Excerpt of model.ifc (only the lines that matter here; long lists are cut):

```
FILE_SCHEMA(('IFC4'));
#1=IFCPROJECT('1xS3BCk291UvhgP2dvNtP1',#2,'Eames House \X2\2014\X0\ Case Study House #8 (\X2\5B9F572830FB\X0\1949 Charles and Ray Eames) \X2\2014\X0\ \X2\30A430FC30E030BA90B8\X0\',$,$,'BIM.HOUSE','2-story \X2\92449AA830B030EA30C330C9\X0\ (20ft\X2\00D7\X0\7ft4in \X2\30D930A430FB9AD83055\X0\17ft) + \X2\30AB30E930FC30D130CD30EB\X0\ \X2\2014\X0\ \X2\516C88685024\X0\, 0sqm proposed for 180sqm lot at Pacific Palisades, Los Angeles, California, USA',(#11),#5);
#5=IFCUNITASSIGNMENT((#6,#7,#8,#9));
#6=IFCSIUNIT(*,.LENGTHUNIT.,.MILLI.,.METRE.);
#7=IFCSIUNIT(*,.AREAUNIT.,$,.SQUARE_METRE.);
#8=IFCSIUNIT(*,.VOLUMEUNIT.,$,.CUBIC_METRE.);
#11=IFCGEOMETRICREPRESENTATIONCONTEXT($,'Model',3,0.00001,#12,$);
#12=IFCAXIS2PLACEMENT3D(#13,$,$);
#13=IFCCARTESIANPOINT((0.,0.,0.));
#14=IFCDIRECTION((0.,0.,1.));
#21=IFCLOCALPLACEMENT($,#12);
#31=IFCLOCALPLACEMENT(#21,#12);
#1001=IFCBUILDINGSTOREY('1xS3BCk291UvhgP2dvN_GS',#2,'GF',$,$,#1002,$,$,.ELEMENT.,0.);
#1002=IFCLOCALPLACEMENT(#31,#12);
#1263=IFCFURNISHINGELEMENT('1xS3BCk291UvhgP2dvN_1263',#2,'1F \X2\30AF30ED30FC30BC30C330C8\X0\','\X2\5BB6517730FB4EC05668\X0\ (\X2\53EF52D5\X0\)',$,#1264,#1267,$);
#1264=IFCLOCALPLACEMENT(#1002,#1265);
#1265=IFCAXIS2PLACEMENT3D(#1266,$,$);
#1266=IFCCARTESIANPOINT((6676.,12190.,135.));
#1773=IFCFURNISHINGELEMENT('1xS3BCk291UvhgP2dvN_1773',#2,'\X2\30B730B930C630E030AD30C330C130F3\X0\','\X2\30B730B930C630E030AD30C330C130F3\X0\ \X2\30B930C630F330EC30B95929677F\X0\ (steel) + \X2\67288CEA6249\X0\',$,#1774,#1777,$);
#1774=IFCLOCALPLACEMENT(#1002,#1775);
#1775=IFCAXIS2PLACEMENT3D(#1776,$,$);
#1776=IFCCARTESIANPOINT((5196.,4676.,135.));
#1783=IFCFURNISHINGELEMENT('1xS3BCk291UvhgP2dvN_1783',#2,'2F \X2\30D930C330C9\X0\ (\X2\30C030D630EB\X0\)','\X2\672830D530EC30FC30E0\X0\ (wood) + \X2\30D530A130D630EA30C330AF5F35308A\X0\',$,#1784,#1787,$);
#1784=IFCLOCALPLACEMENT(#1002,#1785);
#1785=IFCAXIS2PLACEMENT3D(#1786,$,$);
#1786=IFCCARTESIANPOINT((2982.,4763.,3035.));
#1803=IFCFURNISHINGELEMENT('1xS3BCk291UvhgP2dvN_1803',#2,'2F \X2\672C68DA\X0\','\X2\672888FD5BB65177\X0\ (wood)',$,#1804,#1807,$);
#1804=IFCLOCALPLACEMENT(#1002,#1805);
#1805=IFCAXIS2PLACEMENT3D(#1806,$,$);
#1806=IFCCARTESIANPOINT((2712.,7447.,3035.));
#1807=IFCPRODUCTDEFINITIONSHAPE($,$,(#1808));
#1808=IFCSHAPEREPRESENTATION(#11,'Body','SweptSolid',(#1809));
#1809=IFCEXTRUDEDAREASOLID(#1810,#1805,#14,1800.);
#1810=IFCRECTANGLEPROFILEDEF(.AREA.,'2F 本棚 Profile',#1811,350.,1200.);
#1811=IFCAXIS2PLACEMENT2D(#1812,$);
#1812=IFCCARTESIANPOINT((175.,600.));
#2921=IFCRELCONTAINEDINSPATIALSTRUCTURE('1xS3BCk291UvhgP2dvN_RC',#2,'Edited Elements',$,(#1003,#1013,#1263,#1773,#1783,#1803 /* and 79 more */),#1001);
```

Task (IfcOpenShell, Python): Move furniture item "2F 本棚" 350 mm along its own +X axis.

```python
import ifcopenshell
import ifcopenshell.api.geometry
import ifcopenshell.util.placement
import ifcopenshell.util.unit

model = ifcopenshell.open("model.ifc")
unit_scale = ifcopenshell.util.unit.calculate_unit_scale(model)

item = model.by_guid("1xS3BCk291UvhgP2dvN_1803")
matrix = ifcopenshell.util.placement.get_local_placement(item.ObjectPlacement)
matrix[:3, 3] += matrix[:3, 0] * 0.35 / unit_scale
ifcopenshell.api.geometry.edit_object_placement(model, product=item, matrix=matrix, is_si=False)

print(ifcopenshell.util.placement.get_local_placement(item.ObjectPlacement).round(3) + 0.0)

model.write("model_updated.ifc")
```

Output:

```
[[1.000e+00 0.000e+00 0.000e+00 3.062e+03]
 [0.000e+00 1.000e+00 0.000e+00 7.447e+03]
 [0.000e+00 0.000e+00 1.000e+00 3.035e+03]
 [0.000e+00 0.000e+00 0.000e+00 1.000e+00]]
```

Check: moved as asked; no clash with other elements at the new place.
